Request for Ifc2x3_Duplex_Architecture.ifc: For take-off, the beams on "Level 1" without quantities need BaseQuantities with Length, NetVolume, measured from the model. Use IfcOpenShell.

First a look at what the model holds.

```python
import ifcopenshell
import ifcopenshell.util.element
import ifcopenshell.util.unit

model = ifcopenshell.open("Ifc2x3_Duplex_Architecture.ifc")
print(model.schema)
for unit_type in ("LENGTHUNIT", "AREAUNIT", "VOLUMEUNIT"):
    print(unit_type, ifcopenshell.util.unit.calculate_unit_scale(model, unit_type))
storey = next(s for s in model.by_type("IfcBuildingStorey") if s.Name == "Level 1")
beams = [e for e in ifcopenshell.util.element.get_decomposition(storey) if e.is_a("IfcBeam")]
for e in sorted(beams, key=lambda e: e.id()):
    print(e.id(), e.is_a(), e.Name, list(ifcopenshell.util.element.get_psets(e, qtos_only=True)), sep=" | ")
```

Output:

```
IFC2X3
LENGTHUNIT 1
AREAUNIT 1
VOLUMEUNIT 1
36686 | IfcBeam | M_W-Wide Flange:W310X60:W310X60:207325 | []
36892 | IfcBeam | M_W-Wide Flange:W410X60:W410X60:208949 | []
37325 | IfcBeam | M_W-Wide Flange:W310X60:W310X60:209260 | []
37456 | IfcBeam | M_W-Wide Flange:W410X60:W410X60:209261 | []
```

```python
import ifcopenshell
import ifcopenshell.api.pset
import ifcopenshell.geom
import ifcopenshell.util.element
import ifcopenshell.util.shape
import ifcopenshell.util.unit

model = ifcopenshell.open("Ifc2x3_Duplex_Architecture.ifc")
unit_scale = ifcopenshell.util.unit.calculate_unit_scale(model)
volume_scale = ifcopenshell.util.unit.calculate_unit_scale(model, "VOLUMEUNIT")
settings = ifcopenshell.geom.settings()

storey = next(s for s in model.by_type("IfcBuildingStorey") if s.Name == "Level 1")
beams = [e for e in ifcopenshell.util.element.get_decomposition(storey) if e.is_a("IfcBeam")]

for e in sorted(beams, key=lambda e: e.id()):
    if ifcopenshell.util.element.get_psets(e, qtos_only=True, should_inherit=False):
        continue
    # Geometry comes back in metres, in the element's own axes.
    shape = ifcopenshell.geom.create_shape(settings, e)
    values = {
        "Length": ifcopenshell.util.shape.get_max_xyz(shape.geometry) / unit_scale,
        "NetVolume": ifcopenshell.util.shape.get_volume(shape.geometry) / volume_scale,
    }
    qto = ifcopenshell.api.pset.add_qto(model, product=e, name="BaseQuantities")
    ifcopenshell.api.pset.edit_qto(model, qto=qto, properties=values)
    print(e.id(), {k: round(v, 3) for k, v in values.items()})

model.write("Ifc2x3_Duplex_Architecture_v2.ifc")
```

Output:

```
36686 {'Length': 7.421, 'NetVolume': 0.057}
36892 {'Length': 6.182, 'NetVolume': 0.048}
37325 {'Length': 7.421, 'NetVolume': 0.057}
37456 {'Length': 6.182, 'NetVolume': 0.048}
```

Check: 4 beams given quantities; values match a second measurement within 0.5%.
